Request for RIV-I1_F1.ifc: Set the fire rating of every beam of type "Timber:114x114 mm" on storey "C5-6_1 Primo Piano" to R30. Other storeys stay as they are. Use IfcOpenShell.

First a look at what the model holds.

```python
import ifcopenshell
import ifcopenshell.util.element

model = ifcopenshell.open("RIV-I1_F1.ifc")
print(model.schema)
storey = next(s for s in model.by_type("IfcBuildingStorey") if s.Name == "C5-6_1 Primo Piano")
beams = [e for e in ifcopenshell.util.element.get_decomposition(storey) if e.is_a("IfcBeam")]
seen = {}
for e in beams:
    element_type = ifcopenshell.util.element.get_type(e)
    key = (element_type.Name if element_type != e and element_type else None, ifcopenshell.util.element.get_pset(e, "Pset_BeamCommon", "FireRating"))
    seen[key] = seen.get(key, 0) + 1
for (name, value), count in sorted(seen.items(), key=str):
    print(count, "x", name, "|", value)
```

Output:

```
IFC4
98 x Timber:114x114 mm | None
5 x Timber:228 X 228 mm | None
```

```python
import ifcopenshell
import ifcopenshell.api.pset
import ifcopenshell.util.element

model = ifcopenshell.open("RIV-I1_F1.ifc")

storey = next(s for s in model.by_type("IfcBuildingStorey") if s.Name == "C5-6_1 Primo Piano")
beams = [e for e in ifcopenshell.util.element.get_decomposition(storey) if e.is_a("IfcBeam")]

count = 0
for e in beams:
    element_type = ifcopenshell.util.element.get_type(e)
    if element_type in (None, e) or element_type.Name != "Timber:114x114 mm":
        continue
    # add_pset returns the element's existing set when there is one.
    pset = ifcopenshell.api.pset.add_pset(model, product=e, name="Pset_BeamCommon")
    ifcopenshell.api.pset.edit_pset(model, pset=pset, properties={"FireRating": "R30"})
    count += 1

print(count, "beams updated")

model.write("RIV-I1_F1_updated.ifc")
```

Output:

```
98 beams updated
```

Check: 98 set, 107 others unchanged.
